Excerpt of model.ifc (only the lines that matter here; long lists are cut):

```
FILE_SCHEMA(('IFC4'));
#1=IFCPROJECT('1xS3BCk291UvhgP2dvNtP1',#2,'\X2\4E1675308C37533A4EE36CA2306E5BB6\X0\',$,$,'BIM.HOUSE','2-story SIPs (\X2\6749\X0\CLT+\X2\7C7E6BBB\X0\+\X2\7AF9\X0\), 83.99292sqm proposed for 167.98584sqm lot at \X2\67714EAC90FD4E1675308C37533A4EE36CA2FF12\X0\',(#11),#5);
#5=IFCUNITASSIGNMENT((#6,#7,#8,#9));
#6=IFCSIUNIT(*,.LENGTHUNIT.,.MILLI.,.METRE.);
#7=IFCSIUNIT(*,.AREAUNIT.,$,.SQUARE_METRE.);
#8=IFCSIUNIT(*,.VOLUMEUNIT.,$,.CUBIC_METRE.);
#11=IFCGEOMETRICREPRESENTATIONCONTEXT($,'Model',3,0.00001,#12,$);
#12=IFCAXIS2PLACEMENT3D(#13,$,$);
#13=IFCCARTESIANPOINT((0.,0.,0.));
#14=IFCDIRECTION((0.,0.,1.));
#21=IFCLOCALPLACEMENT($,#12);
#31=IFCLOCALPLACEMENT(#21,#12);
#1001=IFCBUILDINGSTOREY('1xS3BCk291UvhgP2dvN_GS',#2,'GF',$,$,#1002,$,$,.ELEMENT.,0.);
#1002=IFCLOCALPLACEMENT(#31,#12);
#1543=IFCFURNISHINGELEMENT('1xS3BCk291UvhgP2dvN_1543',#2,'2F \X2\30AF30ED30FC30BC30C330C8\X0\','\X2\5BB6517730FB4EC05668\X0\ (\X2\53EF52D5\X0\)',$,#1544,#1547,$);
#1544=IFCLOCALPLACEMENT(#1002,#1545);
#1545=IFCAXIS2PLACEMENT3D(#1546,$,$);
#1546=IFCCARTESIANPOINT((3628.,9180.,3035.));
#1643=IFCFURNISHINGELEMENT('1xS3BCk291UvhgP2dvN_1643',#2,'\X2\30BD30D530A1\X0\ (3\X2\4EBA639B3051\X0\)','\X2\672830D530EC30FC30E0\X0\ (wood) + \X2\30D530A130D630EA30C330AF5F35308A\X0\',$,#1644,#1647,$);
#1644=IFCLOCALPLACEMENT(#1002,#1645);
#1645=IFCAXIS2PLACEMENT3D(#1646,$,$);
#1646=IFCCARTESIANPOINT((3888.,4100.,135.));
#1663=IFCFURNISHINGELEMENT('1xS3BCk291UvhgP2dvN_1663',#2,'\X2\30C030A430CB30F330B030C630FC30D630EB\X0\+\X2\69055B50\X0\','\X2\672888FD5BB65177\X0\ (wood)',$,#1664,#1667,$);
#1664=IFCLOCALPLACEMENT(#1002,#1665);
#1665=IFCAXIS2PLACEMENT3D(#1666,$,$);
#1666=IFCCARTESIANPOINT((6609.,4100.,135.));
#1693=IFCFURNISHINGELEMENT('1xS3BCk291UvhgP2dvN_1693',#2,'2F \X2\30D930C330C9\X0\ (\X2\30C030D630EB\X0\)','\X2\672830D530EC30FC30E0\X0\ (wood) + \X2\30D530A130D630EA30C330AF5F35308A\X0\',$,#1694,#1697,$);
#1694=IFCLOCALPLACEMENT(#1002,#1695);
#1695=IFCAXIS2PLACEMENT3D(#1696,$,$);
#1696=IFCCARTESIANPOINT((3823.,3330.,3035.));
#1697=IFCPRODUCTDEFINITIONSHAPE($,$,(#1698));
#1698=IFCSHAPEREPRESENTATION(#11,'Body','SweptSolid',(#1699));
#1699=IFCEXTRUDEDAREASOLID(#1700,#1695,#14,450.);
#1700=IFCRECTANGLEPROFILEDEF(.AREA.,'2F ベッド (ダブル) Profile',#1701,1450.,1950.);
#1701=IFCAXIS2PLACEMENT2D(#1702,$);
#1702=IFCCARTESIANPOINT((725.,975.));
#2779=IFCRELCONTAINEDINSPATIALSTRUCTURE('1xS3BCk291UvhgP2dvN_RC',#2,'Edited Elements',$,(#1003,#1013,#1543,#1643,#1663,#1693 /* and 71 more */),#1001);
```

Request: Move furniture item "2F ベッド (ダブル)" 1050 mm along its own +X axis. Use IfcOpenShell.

```python
import ifcopenshell
import ifcopenshell.api.geometry
import ifcopenshell.util.placement
import ifcopenshell.util.unit

model = ifcopenshell.open("model.ifc")
unit_scale = ifcopenshell.util.unit.calculate_unit_scale(model)

item = model.by_guid("1xS3BCk291UvhgP2dvN_1693")
matrix = ifcopenshell.util.placement.get_local_placement(item.ObjectPlacement)
matrix[:3, 3] += matrix[:3, 0] * 1.05 / unit_scale
ifcopenshell.api.geometry.edit_object_placement(model, product=item, matrix=matrix, is_si=False)

print(ifcopenshell.util.placement.get_local_placement(item.ObjectPlacement).round(3) + 0.0)

model.write("model-out.ifc")
```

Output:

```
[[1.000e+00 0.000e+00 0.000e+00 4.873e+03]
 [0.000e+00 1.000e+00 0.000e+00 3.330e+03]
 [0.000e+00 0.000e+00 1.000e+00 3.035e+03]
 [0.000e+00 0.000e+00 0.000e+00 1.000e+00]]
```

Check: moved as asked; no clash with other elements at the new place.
